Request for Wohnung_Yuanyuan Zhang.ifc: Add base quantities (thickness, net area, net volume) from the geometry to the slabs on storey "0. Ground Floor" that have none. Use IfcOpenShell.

First a look at what the model holds.

```python
import ifcopenshell
import ifcopenshell.util.element
import ifcopenshell.util.unit

model = ifcopenshell.open("Wohnung_Yuanyuan Zhang.ifc")
print(model.schema)
for unit_type in ("LENGTHUNIT", "AREAUNIT", "VOLUMEUNIT"):
    print(unit_type, ifcopenshell.util.unit.calculate_unit_scale(model, unit_type))
storey = next(s for s in model.by_type("IfcBuildingStorey") if s.Name == "0. Ground Floor")
slabs = [e for e in ifcopenshell.util.element.get_decomposition(storey) if e.is_a("IfcSlab")]
for e in sorted(slabs, key=lambda e: e.id()):
    print(e.id(), e.is_a(), e.Name, list(ifcopenshell.util.element.get_psets(e, qtos_only=True)), sep=" | ")
```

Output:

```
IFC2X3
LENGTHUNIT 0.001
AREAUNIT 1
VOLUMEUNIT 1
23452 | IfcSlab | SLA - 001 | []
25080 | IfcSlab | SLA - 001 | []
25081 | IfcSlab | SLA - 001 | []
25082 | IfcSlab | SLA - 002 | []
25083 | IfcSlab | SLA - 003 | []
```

```python
import ifcopenshell
import ifcopenshell.api.pset
import ifcopenshell.geom
import ifcopenshell.util.element
import ifcopenshell.util.shape
import ifcopenshell.util.unit

model = ifcopenshell.open("Wohnung_Yuanyuan Zhang.ifc")
unit_scale = ifcopenshell.util.unit.calculate_unit_scale(model)
area_scale = ifcopenshell.util.unit.calculate_unit_scale(model, "AREAUNIT")
volume_scale = ifcopenshell.util.unit.calculate_unit_scale(model, "VOLUMEUNIT")
settings = ifcopenshell.geom.settings()

storey = next(s for s in model.by_type("IfcBuildingStorey") if s.Name == "0. Ground Floor")
slabs = [e for e in ifcopenshell.util.element.get_decomposition(storey) if e.is_a("IfcSlab")]

for e in sorted(slabs, key=lambda e: e.id()):
    if ifcopenshell.util.element.get_psets(e, qtos_only=True, should_inherit=False):
        continue
    # Geometry comes back in metres, in the element's own axes.
    shape = ifcopenshell.geom.create_shape(settings, e)
    values = {
        "Width": ifcopenshell.util.shape.get_z(shape.geometry) / unit_scale,
        "NetArea": ifcopenshell.util.shape.get_footprint_area(shape.geometry) / area_scale,
        "NetVolume": ifcopenshell.util.shape.get_volume(shape.geometry) / volume_scale,
    }
    qto = ifcopenshell.api.pset.add_qto(model, product=e, name="BaseQuantities")
    ifcopenshell.api.pset.edit_qto(model, qto=qto, properties=values)
    print(e.id(), {k: round(v, 3) for k, v in values.items()})

model.write("Wohnung_Yuanyuan Zhang_edited.ifc")
```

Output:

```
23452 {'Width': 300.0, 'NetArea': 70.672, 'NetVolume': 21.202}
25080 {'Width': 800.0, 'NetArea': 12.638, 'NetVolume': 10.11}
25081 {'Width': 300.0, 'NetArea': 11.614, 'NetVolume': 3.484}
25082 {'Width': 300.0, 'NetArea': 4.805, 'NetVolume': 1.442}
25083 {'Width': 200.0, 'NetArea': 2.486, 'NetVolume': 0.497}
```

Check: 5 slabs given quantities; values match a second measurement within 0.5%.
